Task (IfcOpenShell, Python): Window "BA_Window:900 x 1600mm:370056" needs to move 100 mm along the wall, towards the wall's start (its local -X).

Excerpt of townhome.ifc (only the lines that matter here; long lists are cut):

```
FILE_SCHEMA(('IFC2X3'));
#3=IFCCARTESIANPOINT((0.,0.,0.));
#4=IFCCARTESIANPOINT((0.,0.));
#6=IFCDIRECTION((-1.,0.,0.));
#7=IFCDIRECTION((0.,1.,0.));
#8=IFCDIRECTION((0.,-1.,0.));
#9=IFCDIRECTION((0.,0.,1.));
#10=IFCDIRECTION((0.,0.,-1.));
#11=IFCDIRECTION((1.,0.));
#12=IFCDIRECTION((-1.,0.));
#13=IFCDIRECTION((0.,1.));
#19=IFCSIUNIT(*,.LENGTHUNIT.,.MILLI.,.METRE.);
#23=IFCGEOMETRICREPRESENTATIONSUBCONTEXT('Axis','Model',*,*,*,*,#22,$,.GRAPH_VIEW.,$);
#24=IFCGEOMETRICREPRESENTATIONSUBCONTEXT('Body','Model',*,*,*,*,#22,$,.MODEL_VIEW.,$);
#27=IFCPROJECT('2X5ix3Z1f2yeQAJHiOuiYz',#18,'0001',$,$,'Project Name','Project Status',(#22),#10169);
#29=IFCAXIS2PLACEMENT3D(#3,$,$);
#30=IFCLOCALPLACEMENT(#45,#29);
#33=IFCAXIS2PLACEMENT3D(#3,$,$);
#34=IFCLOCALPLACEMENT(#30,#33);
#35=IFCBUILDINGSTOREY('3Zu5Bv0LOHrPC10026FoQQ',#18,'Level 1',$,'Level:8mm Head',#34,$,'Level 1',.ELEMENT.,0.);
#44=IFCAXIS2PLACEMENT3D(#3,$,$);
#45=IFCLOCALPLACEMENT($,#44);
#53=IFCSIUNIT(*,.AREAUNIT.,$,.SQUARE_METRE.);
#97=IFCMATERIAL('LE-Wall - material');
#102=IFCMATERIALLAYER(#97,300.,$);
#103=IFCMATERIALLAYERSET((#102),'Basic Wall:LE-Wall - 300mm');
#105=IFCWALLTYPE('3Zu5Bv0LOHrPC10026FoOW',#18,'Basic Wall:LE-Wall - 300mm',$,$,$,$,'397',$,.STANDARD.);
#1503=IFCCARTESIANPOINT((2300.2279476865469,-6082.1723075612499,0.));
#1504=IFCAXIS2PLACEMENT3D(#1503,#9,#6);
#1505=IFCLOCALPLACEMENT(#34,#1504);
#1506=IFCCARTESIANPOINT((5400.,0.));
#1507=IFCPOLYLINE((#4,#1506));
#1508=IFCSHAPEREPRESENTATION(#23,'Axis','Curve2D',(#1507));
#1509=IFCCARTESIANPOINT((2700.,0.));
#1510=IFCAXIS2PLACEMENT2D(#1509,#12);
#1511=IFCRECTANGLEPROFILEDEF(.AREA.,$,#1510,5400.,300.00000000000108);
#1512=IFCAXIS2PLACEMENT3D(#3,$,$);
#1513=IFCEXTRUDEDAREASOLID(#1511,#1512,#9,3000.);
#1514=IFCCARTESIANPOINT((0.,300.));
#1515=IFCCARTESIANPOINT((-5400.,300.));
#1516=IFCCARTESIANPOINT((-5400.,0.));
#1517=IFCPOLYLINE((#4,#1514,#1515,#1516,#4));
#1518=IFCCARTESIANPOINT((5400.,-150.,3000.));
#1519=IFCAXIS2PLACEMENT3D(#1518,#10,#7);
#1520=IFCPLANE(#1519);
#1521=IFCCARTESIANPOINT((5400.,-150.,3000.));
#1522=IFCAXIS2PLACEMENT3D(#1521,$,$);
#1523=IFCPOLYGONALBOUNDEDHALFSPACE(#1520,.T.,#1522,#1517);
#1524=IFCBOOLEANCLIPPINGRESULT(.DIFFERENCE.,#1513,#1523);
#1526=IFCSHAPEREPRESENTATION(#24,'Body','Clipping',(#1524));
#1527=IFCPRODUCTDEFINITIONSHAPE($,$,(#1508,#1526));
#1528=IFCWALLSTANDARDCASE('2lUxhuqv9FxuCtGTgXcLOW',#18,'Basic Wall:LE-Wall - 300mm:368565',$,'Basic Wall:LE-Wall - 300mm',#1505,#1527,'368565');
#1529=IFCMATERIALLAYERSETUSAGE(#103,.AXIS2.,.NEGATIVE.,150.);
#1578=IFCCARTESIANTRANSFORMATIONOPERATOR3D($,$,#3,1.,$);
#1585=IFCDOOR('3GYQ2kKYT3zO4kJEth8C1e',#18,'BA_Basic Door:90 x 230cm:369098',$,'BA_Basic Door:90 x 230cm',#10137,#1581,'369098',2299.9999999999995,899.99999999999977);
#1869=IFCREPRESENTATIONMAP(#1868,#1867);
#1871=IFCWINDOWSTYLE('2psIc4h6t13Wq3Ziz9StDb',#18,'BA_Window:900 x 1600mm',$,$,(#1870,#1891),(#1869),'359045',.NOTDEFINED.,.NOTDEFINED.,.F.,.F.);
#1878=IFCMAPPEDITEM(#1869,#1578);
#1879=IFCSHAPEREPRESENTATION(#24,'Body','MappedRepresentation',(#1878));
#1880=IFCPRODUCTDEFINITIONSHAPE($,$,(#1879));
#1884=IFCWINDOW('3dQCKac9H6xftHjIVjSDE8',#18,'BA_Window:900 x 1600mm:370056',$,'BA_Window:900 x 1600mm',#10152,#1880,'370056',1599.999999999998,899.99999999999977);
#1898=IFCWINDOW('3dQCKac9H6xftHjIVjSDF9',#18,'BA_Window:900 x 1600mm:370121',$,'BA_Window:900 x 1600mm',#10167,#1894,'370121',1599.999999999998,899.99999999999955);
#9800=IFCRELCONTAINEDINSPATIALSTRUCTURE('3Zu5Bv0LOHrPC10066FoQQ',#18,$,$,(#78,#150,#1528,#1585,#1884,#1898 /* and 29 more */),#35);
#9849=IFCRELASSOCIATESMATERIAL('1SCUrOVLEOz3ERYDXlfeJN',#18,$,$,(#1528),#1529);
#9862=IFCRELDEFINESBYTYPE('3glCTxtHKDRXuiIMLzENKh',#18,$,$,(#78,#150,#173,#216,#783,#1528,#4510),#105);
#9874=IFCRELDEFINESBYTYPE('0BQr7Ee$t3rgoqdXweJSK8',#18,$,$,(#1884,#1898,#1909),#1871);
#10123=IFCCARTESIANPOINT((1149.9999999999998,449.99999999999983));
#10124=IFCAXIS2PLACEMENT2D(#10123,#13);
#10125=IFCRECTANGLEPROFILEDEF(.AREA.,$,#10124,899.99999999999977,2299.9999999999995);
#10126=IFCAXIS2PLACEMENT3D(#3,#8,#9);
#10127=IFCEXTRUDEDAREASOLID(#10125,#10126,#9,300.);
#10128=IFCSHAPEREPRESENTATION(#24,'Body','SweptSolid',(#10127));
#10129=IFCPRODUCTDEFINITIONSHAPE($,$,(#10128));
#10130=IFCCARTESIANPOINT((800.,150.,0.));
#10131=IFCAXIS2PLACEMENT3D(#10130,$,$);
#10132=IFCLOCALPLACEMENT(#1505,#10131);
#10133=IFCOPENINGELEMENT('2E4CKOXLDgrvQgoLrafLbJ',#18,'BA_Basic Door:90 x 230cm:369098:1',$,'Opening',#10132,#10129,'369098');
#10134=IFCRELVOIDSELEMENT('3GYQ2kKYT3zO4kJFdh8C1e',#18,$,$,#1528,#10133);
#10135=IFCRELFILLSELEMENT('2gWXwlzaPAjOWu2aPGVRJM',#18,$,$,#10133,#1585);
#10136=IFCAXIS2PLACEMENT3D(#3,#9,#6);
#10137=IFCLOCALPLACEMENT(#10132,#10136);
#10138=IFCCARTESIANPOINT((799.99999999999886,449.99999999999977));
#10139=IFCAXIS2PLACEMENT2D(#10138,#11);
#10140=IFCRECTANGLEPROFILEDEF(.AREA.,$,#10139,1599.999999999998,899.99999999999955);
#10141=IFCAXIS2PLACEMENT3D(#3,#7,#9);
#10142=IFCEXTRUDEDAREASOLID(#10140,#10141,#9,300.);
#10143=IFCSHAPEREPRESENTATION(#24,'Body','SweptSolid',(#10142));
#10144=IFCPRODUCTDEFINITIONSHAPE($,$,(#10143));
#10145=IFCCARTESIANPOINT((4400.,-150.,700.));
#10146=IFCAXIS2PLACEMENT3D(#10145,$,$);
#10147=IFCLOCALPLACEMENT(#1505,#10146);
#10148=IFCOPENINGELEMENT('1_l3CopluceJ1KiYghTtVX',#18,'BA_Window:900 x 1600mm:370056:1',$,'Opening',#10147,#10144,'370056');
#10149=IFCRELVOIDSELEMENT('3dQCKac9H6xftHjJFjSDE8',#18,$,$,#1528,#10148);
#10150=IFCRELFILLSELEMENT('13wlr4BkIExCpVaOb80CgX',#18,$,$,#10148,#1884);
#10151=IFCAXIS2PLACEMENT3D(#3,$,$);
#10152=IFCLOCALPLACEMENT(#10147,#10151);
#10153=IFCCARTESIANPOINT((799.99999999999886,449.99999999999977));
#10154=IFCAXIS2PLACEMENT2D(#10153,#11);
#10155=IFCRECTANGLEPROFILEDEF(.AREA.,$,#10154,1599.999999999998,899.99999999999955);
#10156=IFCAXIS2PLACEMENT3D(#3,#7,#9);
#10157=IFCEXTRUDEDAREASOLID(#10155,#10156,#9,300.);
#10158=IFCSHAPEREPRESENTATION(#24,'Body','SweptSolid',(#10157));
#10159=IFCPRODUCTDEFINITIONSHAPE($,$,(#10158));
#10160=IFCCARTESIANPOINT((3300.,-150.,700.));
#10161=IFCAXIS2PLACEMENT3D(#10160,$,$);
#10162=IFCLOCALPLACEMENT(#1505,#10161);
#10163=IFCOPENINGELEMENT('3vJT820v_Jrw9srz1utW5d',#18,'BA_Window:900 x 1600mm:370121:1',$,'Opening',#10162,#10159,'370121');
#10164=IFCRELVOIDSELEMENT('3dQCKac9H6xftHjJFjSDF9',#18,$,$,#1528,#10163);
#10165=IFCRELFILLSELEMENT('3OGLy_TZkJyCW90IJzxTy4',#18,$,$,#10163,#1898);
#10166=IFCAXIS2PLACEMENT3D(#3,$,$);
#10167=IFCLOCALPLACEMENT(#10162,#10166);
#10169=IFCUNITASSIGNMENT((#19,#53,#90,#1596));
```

```python
import ifcopenshell
import ifcopenshell.api.geometry
import ifcopenshell.util.placement
import ifcopenshell.util.unit

model = ifcopenshell.open("townhome.ifc")
unit_scale = ifcopenshell.util.unit.calculate_unit_scale(model)

window = model.by_guid("3dQCKac9H6xftHjIVjSDE8")
opening = window.FillsVoids[0].RelatingOpeningElement
wall = opening.VoidsElements[0].RelatingBuildingElement

wall_matrix = ifcopenshell.util.placement.get_local_placement(wall.ObjectPlacement)
shift = wall_matrix[:3, 0] * -0.1 / unit_scale
before = ifcopenshell.util.placement.get_local_placement(window.ObjectPlacement)[:3, 3].copy()

# The window is placed relative to its opening, so it follows when the opening moves.
matrix = ifcopenshell.util.placement.get_local_placement(opening.ObjectPlacement)
matrix[:3, 3] += shift
ifcopenshell.api.geometry.edit_object_placement(
    model, product=opening, matrix=matrix, is_si=False, should_transform_children=True
)

after = ifcopenshell.util.placement.get_local_placement(window.ObjectPlacement)[:3, 3]
print("window moved by", (after - before).round(3) + 0.0)

model.write("townhome-out.ifc")
```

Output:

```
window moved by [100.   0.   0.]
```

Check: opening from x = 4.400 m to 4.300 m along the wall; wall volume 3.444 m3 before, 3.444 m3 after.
